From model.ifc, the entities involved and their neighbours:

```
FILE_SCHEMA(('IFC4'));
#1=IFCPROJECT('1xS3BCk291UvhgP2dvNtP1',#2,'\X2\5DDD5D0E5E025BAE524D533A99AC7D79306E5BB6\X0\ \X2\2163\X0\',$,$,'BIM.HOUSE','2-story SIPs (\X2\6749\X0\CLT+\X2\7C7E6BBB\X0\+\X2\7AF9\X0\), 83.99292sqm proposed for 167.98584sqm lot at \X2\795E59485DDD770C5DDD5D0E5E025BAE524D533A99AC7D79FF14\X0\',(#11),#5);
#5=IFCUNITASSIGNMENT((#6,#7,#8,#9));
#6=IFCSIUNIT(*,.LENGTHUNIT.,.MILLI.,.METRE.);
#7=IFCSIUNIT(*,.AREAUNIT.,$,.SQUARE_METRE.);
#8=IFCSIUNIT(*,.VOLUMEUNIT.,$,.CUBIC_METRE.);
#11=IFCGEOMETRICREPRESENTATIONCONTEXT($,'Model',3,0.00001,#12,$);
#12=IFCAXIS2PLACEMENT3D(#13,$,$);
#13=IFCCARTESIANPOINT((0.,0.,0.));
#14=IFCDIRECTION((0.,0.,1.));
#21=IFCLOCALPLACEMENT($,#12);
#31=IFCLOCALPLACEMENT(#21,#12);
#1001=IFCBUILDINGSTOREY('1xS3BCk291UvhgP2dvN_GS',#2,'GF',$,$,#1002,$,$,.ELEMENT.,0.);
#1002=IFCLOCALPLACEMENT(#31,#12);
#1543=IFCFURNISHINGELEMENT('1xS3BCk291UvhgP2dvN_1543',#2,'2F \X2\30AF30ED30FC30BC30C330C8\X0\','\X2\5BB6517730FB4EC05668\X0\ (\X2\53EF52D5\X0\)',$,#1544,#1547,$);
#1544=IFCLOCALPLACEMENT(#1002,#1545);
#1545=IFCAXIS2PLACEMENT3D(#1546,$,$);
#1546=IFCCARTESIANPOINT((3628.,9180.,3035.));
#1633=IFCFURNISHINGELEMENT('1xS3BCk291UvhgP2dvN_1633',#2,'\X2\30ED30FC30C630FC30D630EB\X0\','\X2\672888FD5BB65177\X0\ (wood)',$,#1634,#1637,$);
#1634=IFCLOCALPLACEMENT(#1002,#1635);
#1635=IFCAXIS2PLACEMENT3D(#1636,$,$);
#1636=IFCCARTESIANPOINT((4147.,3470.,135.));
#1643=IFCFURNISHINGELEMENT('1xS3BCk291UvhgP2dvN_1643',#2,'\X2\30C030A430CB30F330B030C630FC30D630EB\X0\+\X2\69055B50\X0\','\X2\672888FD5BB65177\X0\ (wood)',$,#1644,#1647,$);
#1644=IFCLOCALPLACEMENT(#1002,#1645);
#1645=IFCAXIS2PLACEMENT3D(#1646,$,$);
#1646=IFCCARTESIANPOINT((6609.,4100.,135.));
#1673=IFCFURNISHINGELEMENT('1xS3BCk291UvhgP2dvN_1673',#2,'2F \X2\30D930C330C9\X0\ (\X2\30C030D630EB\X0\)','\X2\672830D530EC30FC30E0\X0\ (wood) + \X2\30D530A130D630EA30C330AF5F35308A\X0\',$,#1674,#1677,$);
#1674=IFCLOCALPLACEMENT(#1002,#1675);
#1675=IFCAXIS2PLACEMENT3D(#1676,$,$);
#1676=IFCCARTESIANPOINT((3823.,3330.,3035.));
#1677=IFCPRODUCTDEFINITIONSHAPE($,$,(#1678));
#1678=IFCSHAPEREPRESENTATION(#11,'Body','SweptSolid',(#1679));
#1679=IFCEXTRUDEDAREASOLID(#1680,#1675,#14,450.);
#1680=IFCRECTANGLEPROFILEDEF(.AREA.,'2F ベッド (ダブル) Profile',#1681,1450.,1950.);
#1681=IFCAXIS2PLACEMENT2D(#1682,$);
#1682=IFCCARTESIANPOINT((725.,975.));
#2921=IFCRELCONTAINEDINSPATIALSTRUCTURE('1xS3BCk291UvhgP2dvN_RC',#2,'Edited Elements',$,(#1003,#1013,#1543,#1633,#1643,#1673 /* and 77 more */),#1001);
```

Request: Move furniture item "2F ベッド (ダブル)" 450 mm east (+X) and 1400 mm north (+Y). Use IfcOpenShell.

```python
import ifcopenshell
import ifcopenshell.api.geometry
import ifcopenshell.util.placement

model = ifcopenshell.open("model.ifc")

item = model.by_guid("1xS3BCk291UvhgP2dvN_1673")
matrix = ifcopenshell.util.placement.get_local_placement(item.ObjectPlacement)
matrix[0, 3] += 450.0
matrix[1, 3] += 1400.0
ifcopenshell.api.geometry.edit_object_placement(model, product=item, matrix=matrix, is_si=False)

print(ifcopenshell.util.placement.get_local_placement(item.ObjectPlacement).round(3) + 0.0)

model.write("model-out.ifc")
```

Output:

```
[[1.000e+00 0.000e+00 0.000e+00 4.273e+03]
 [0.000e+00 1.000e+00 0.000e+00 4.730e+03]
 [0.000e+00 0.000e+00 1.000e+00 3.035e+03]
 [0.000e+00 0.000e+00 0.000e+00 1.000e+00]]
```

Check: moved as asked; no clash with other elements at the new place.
